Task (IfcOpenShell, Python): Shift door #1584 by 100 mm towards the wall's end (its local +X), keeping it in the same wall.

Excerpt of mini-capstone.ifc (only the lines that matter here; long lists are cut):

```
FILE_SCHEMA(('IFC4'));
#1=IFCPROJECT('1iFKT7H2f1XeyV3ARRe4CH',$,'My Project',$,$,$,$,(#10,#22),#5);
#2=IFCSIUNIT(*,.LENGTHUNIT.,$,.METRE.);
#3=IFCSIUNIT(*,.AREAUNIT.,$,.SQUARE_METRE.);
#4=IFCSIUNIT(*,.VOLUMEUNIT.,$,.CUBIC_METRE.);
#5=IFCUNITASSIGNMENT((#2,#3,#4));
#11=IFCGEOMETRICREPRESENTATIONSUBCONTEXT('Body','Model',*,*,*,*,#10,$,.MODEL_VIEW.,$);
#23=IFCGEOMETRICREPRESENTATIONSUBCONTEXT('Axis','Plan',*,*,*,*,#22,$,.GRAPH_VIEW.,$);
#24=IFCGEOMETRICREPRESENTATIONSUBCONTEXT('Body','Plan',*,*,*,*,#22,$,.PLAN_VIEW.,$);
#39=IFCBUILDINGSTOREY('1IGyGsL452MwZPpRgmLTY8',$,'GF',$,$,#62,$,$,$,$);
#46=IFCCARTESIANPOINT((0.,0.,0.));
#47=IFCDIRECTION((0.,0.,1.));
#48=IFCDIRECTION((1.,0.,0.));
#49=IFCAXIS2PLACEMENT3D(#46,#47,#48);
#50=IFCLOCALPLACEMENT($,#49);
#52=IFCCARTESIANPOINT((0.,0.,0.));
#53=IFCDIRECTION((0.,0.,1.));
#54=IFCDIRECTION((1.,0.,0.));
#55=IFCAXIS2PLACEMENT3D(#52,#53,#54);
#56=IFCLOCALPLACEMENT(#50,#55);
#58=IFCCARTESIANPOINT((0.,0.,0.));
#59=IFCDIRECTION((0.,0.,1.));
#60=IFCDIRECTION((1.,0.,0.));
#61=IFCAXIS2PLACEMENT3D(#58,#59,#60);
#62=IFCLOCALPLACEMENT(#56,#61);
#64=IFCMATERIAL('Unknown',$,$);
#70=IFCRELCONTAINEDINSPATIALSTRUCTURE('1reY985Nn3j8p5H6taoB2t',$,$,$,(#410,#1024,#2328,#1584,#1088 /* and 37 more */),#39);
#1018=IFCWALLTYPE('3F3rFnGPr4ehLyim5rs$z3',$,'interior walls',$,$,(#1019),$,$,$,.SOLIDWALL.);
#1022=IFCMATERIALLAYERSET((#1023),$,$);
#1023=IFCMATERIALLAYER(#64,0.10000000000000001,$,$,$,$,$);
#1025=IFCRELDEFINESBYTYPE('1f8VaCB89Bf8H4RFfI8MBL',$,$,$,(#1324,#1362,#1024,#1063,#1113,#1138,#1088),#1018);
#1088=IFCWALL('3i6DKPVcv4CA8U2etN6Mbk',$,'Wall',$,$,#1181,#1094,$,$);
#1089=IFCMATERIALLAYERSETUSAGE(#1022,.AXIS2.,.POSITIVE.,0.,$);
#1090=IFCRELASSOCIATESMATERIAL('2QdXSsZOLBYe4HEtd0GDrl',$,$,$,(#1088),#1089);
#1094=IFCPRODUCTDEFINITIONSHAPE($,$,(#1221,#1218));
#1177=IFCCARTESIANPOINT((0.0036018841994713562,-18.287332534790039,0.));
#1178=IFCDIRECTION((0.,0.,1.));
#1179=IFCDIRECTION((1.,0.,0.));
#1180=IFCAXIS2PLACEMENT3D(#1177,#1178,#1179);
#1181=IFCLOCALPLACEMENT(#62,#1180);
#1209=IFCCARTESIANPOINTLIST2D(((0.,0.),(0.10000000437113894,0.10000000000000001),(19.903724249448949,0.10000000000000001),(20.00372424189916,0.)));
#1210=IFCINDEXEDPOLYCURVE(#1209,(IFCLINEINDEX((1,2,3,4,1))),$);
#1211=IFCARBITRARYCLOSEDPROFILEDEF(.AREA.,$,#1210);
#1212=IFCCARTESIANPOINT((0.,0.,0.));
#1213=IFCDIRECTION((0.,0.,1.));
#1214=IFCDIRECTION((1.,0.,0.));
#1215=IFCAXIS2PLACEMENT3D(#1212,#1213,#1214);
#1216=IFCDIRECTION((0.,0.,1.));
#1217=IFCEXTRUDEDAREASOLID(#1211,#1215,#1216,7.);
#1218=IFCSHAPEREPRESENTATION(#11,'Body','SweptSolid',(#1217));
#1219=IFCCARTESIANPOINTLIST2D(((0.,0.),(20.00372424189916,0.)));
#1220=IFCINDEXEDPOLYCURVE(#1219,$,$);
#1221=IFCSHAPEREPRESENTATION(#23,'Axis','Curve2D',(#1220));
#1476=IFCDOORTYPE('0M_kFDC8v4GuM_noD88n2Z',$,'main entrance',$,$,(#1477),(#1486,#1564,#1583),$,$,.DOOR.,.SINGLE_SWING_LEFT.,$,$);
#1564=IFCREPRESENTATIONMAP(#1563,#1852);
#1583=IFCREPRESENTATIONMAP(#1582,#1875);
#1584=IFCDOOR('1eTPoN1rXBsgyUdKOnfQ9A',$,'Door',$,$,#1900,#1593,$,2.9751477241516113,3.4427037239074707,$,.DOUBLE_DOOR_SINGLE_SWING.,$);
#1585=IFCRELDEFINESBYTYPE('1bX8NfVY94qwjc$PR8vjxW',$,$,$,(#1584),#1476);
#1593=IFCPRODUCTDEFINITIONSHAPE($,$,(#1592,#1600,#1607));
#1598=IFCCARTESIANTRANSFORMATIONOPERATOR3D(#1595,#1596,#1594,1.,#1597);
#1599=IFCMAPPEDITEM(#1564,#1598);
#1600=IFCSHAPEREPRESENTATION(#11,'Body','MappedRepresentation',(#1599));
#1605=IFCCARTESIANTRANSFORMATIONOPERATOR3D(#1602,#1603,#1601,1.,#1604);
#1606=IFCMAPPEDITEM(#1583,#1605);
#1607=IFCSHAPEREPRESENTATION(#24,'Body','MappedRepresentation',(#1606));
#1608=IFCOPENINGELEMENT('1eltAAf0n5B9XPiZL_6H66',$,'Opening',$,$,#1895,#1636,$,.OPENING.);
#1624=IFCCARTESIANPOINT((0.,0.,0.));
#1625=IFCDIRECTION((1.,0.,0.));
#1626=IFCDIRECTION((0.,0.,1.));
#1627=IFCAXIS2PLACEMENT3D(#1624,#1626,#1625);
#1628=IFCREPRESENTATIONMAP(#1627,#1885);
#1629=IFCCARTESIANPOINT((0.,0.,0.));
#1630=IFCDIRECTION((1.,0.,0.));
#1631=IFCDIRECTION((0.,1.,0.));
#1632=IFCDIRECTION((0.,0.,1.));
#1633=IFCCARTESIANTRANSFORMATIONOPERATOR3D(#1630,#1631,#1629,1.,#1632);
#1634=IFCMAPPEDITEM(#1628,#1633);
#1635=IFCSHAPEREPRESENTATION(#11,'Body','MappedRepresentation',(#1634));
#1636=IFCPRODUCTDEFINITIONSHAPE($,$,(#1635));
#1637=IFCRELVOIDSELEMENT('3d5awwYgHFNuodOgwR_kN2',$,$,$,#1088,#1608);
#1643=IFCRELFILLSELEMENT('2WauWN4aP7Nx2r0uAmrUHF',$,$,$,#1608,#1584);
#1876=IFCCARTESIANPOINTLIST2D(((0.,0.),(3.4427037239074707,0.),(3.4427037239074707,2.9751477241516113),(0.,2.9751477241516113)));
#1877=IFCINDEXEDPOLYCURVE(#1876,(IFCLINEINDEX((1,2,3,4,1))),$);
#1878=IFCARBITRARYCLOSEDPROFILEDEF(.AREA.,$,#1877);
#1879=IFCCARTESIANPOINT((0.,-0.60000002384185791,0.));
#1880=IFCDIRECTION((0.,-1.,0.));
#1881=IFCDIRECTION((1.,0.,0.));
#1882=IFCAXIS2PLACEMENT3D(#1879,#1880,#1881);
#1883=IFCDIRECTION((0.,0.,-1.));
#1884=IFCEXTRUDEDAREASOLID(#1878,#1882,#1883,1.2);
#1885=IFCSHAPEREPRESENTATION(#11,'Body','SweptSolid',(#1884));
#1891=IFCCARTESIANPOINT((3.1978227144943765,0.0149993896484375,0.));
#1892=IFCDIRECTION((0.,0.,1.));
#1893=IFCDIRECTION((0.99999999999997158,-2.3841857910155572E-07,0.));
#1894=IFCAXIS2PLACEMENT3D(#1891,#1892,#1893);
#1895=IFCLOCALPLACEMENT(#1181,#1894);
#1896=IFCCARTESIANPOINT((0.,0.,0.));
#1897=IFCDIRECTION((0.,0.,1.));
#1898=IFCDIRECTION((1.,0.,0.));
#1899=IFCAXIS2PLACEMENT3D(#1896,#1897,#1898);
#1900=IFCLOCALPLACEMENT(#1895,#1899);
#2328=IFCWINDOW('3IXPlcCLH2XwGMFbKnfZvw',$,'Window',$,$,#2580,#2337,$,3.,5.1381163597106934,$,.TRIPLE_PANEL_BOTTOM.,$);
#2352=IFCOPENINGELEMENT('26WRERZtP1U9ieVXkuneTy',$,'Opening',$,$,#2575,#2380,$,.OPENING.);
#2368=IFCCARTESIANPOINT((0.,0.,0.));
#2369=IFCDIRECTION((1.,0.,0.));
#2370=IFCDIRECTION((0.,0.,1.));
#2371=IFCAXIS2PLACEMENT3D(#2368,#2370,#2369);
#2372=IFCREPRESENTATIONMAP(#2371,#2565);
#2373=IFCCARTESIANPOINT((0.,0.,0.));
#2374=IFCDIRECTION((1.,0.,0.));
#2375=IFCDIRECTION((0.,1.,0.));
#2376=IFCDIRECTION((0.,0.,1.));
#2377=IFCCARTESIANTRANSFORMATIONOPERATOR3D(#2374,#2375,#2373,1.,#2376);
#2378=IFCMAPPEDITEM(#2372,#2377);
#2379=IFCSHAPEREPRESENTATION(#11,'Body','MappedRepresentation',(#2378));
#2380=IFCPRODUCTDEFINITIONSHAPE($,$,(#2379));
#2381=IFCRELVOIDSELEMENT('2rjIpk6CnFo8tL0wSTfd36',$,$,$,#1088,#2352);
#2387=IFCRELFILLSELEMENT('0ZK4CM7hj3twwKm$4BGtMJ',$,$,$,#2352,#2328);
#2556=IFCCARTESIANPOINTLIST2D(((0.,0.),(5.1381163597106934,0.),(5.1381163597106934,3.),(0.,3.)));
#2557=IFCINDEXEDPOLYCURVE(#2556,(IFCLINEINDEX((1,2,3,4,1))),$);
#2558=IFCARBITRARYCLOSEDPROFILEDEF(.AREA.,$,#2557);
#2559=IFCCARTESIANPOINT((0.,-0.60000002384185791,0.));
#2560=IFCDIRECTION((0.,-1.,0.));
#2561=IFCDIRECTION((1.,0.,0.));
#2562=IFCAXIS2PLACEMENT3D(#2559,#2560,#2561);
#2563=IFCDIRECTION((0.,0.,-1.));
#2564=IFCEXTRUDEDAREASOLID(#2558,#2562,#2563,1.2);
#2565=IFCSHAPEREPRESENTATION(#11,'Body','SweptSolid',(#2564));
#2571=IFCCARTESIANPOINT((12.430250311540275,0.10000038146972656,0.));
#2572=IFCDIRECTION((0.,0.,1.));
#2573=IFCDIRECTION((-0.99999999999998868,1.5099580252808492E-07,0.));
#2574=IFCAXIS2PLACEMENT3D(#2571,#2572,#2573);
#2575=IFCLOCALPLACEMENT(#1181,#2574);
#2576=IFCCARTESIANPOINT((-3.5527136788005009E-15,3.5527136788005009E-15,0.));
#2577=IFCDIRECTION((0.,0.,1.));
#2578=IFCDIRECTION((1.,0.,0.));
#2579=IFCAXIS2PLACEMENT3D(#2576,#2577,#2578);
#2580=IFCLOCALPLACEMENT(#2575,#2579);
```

```python
import ifcopenshell
import ifcopenshell.api.geometry
import ifcopenshell.util.placement
import ifcopenshell.util.unit

model = ifcopenshell.open("mini-capstone.ifc")
unit_scale = ifcopenshell.util.unit.calculate_unit_scale(model)

door = model.by_guid("1eTPoN1rXBsgyUdKOnfQ9A")
opening = door.FillsVoids[0].RelatingOpeningElement
wall = opening.VoidsElements[0].RelatingBuildingElement

wall_matrix = ifcopenshell.util.placement.get_local_placement(wall.ObjectPlacement)
shift = wall_matrix[:3, 0] * 0.1 / unit_scale
before = ifcopenshell.util.placement.get_local_placement(door.ObjectPlacement)[:3, 3].copy()

# The door is placed relative to its opening, so it follows when the opening moves.
matrix = ifcopenshell.util.placement.get_local_placement(opening.ObjectPlacement)
matrix[:3, 3] += shift
ifcopenshell.api.geometry.edit_object_placement(
    model, product=opening, matrix=matrix, is_si=False, should_transform_children=True
)

after = ifcopenshell.util.placement.get_local_placement(door.ObjectPlacement)[:3, 3]
print("door moved by", (after - before).round(3) + 0.0)

model.write("mini-capstone_rev.ifc")
```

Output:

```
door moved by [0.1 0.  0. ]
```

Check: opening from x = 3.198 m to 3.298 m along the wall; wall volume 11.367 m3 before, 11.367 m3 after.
